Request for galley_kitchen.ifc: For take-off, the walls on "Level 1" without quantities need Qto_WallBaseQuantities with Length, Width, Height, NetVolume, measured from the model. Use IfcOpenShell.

First a look at what the model holds.

```python
import ifcopenshell
import ifcopenshell.util.element
import ifcopenshell.util.unit

model = ifcopenshell.open("galley_kitchen.ifc")
print(model.schema)
for unit_type in ("LENGTHUNIT", "AREAUNIT", "VOLUMEUNIT"):
    print(unit_type, ifcopenshell.util.unit.calculate_unit_scale(model, unit_type))
storey = next(s for s in model.by_type("IfcBuildingStorey") if s.Name == "Level 1")
walls = [e for e in ifcopenshell.util.element.get_decomposition(storey) if e.is_a("IfcWall")]
for e in sorted(walls, key=lambda e: e.id()):
    print(e.id(), e.is_a(), e.Name, list(ifcopenshell.util.element.get_psets(e, qtos_only=True)), sep=" | ")
```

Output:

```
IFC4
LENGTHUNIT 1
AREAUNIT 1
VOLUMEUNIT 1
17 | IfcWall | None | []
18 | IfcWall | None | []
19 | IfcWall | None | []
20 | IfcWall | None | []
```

```python
import ifcopenshell
import ifcopenshell.api.pset
import ifcopenshell.geom
import ifcopenshell.util.element
import ifcopenshell.util.shape
import ifcopenshell.util.unit

model = ifcopenshell.open("galley_kitchen.ifc")
unit_scale = ifcopenshell.util.unit.calculate_unit_scale(model)
volume_scale = ifcopenshell.util.unit.calculate_unit_scale(model, "VOLUMEUNIT")
settings = ifcopenshell.geom.settings()

storey = next(s for s in model.by_type("IfcBuildingStorey") if s.Name == "Level 1")
walls = [e for e in ifcopenshell.util.element.get_decomposition(storey) if e.is_a("IfcWall")]

for e in sorted(walls, key=lambda e: e.id()):
    if ifcopenshell.util.element.get_psets(e, qtos_only=True, should_inherit=False):
        continue
    # Geometry comes back in metres, in the element's own axes.
    shape = ifcopenshell.geom.create_shape(settings, e)
    values = {
        "Length": ifcopenshell.util.shape.get_x(shape.geometry) / unit_scale,
        "Width": ifcopenshell.util.shape.get_y(shape.geometry) / unit_scale,
        "Height": ifcopenshell.util.shape.get_z(shape.geometry) / unit_scale,
        "NetVolume": ifcopenshell.util.shape.get_volume(shape.geometry) / volume_scale,
    }
    qto = ifcopenshell.api.pset.add_qto(model, product=e, name="Qto_WallBaseQuantities")
    ifcopenshell.api.pset.edit_qto(model, qto=qto, properties=values)
    print(e.id(), {k: round(v, 3) for k, v in values.items()})

model.write("galley_kitchen_v2.ifc")
```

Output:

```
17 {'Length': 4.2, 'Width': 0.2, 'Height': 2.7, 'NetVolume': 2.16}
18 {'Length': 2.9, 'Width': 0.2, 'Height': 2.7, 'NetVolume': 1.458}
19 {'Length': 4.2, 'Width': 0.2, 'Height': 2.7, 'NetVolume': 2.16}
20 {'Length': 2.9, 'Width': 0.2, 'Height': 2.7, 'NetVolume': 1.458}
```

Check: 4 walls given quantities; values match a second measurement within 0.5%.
